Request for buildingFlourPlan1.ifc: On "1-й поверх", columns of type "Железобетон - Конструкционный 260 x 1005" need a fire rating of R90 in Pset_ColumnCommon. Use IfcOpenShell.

First a look at what the model holds.

```python
import ifcopenshell
import ifcopenshell.util.element

model = ifcopenshell.open("buildingFlourPlan1.ifc")
print(model.schema)
storey = next(s for s in model.by_type("IfcBuildingStorey") if s.Name == "1-й поверх")
columns = [e for e in ifcopenshell.util.element.get_decomposition(storey) if e.is_a("IfcColumn")]
seen = {}
for e in columns:
    element_type = ifcopenshell.util.element.get_type(e)
    key = (element_type.Name if element_type != e and element_type else None, ifcopenshell.util.element.get_pset(e, "Pset_ColumnCommon", "FireRating"))
    seen[key] = seen.get(key, 0) + 1
for (name, value), count in sorted(seen.items(), key=str):
    print(count, "x", name, "|", value)
```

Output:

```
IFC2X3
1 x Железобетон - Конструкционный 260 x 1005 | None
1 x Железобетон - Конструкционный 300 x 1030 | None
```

```python
import ifcopenshell
import ifcopenshell.api.pset
import ifcopenshell.util.element

model = ifcopenshell.open("buildingFlourPlan1.ifc")

storey = next(s for s in model.by_type("IfcBuildingStorey") if s.Name == "1-й поверх")
columns = [e for e in ifcopenshell.util.element.get_decomposition(storey) if e.is_a("IfcColumn")]

count = 0
for e in columns:
    element_type = ifcopenshell.util.element.get_type(e)
    if element_type in (None, e) or element_type.Name != "Железобетон - Конструкционный 260 x 1005":
        continue
    # add_pset returns the element's existing set when there is one.
    pset = ifcopenshell.api.pset.add_pset(model, product=e, name="Pset_ColumnCommon")
    ifcopenshell.api.pset.edit_pset(model, pset=pset, properties={"FireRating": "R90"})
    count += 1

print(count, "columns updated")

model.write("buildingFlourPlan1_rev.ifc")
```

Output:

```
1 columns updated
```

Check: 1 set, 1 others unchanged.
